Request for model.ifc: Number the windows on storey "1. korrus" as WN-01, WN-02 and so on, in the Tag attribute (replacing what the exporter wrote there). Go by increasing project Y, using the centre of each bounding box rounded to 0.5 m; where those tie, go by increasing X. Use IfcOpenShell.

First a look at what the model holds.

```python
import ifcopenshell
import ifcopenshell.util.element
import ifcopenshell.util.placement

model = ifcopenshell.open("model.ifc")
print(model.schema)
storey = next(s for s in model.by_type("IfcBuildingStorey") if s.Name == "1. korrus")
windows = [e for e in ifcopenshell.util.element.get_decomposition(storey) if e.is_a("IfcWindow")]
for e in sorted(windows, key=lambda e: e.id()):
    origin = ifcopenshell.util.placement.get_local_placement(e.ObjectPlacement)[:3, 3]
    print(e.id(), e.Tag, e.Name, origin.round(2) + 0.0, sep=" | ")
```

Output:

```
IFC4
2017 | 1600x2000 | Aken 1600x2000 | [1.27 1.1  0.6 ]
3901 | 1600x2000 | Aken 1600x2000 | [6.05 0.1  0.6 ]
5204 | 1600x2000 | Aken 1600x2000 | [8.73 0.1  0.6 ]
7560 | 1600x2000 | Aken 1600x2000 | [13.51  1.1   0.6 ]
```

```python
import ifcopenshell
import ifcopenshell.geom
import ifcopenshell.util.element
import ifcopenshell.util.shape

model = ifcopenshell.open("model.ifc")
settings = ifcopenshell.geom.settings()
settings.set("use-world-coords", True)


def centre(element):
    shape = ifcopenshell.geom.create_shape(settings, element)
    return ifcopenshell.util.shape.get_bbox_centroid(shape.geometry)


storey = next(s for s in model.by_type("IfcBuildingStorey") if s.Name == "1. korrus")
windows = [e for e in ifcopenshell.util.element.get_decomposition(storey) if e.is_a("IfcWindow")]

# Insertion points can sit at a corner or the storey origin, so sort by the geometry (in metres).
centres = {e: centre(e) for e in windows}
windows.sort(key=lambda e: (round(centres[e][1] / 0.5), centres[e][0]))

for i, e in enumerate(windows, start=1):
    number = f"WN-{i:02d}"
    e.Tag = number
    print(e.id(), number)

model.write("model_updated.ifc")
```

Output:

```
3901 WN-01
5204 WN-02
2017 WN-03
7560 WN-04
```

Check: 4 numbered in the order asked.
